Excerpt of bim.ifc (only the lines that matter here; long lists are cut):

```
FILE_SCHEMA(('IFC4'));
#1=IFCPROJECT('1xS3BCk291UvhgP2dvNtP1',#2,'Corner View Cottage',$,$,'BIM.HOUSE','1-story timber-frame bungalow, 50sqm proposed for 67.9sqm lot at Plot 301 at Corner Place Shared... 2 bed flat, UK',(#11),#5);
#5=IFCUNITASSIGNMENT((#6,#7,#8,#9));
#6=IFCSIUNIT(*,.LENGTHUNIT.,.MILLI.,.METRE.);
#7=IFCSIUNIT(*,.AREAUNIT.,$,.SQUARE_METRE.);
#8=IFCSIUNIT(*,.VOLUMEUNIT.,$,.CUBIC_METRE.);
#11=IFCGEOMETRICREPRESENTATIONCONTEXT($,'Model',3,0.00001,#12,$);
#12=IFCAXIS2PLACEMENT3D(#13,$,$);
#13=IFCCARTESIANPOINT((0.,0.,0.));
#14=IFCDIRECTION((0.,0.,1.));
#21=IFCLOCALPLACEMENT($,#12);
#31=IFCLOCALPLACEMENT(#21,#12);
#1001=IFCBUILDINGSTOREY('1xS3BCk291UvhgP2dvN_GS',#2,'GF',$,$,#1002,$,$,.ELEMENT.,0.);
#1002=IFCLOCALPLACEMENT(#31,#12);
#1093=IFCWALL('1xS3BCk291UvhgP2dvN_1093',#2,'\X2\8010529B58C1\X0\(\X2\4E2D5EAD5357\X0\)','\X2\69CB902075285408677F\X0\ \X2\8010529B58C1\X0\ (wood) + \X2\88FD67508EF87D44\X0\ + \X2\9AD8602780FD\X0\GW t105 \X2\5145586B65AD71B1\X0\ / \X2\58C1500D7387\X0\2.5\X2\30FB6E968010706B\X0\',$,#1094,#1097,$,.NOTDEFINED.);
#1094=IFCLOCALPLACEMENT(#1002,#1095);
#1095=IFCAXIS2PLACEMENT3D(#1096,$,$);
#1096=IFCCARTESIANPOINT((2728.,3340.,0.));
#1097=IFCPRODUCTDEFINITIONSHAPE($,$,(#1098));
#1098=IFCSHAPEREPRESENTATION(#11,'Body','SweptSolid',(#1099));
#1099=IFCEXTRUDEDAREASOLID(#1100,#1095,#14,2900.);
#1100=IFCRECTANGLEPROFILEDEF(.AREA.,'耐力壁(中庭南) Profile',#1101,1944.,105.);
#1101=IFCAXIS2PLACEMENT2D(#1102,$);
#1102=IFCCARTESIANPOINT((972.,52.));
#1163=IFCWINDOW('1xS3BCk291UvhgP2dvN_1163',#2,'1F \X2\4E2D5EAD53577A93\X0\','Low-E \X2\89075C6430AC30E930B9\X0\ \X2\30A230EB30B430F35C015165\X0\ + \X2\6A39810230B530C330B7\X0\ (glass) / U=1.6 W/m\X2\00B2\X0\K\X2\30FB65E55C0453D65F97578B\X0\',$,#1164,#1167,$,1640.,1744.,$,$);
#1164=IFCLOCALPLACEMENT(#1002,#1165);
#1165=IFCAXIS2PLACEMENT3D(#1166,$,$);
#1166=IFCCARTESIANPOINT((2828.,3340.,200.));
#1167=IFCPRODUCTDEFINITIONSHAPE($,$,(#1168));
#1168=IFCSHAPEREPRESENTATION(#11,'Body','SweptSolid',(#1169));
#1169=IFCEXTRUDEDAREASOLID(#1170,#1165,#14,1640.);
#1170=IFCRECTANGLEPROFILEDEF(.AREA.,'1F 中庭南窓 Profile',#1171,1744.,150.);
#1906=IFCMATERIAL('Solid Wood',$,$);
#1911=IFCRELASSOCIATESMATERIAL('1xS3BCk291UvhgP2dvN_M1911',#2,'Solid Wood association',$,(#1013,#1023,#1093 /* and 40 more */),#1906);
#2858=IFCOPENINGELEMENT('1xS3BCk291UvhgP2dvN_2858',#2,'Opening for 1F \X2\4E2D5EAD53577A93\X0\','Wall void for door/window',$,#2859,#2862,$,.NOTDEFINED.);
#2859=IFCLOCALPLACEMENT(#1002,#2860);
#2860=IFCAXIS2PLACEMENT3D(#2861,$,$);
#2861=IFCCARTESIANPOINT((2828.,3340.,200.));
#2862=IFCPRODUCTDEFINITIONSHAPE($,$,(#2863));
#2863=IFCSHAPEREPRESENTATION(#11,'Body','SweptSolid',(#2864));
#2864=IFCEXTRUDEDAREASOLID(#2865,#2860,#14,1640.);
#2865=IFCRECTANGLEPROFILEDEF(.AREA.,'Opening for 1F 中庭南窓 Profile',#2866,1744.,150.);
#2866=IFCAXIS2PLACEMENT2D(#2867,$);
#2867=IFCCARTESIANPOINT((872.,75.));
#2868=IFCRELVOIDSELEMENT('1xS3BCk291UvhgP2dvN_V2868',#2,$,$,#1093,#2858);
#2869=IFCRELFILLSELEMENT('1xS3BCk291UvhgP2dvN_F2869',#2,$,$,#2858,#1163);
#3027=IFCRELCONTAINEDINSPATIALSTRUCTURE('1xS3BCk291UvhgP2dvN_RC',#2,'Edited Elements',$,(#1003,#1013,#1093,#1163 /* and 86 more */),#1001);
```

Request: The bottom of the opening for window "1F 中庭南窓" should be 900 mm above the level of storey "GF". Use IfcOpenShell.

```python
import numpy as np
import ifcopenshell
import ifcopenshell.api.geometry
import ifcopenshell.geom
import ifcopenshell.util.element
import ifcopenshell.util.placement
import ifcopenshell.util.shape
import ifcopenshell.util.unit

model = ifcopenshell.open("bim.ifc")
unit_scale = ifcopenshell.util.unit.calculate_unit_scale(model)

window = model.by_guid("1xS3BCk291UvhgP2dvN_1163")
opening = window.FillsVoids[0].RelatingOpeningElement
storey = ifcopenshell.util.element.get_container(window, ifc_class="IfcBuildingStorey")
level = ifcopenshell.util.placement.get_local_placement(storey.ObjectPlacement)[2, 3]

# The opening's origin need not be at the sill, so measure its lowest point.
shape = ifcopenshell.geom.create_shape(ifcopenshell.geom.settings(), opening)
bottom = ifcopenshell.util.shape.get_shape_bottom_elevation(shape, shape.geometry) / unit_scale
dz = level + 900.0 - bottom

shift = np.array([0.0, 0.0, dz])
# The window is not placed relative to its opening, so move both.
for product in (opening, window):
    matrix = ifcopenshell.util.placement.get_local_placement(product.ObjectPlacement)
    matrix[:3, 3] += shift
    ifcopenshell.api.geometry.edit_object_placement(model, product=product, matrix=matrix, is_si=False)

print(f"moved by {dz * unit_scale:+.3f} m")

model.write("bim_edited.ifc")
```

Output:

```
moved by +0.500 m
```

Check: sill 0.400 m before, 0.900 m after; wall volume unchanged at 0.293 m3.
